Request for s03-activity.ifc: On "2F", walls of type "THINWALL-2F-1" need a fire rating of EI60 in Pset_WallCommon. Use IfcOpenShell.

First a look at what the model holds.

```python
import ifcopenshell
import ifcopenshell.util.element

model = ifcopenshell.open("s03-activity.ifc")
print(model.schema)
storey = next(s for s in model.by_type("IfcBuildingStorey") if s.Name == "2F")
walls = [e for e in ifcopenshell.util.element.get_decomposition(storey) if e.is_a("IfcWall")]
seen = {}
for e in walls:
    element_type = ifcopenshell.util.element.get_type(e)
    key = (element_type.Name if element_type != e and element_type else None, ifcopenshell.util.element.get_pset(e, "Pset_WallCommon", "FireRating"))
    seen[key] = seen.get(key, 0) + 1
for (name, value), count in sorted(seen.items(), key=str):
    print(count, "x", name, "|", value)
```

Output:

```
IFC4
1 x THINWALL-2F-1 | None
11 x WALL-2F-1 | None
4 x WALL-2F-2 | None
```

```python
import ifcopenshell
import ifcopenshell.api.pset
import ifcopenshell.util.element

model = ifcopenshell.open("s03-activity.ifc")

storey = next(s for s in model.by_type("IfcBuildingStorey") if s.Name == "2F")
walls = [e for e in ifcopenshell.util.element.get_decomposition(storey) if e.is_a("IfcWall")]

count = 0
for e in walls:
    element_type = ifcopenshell.util.element.get_type(e)
    if element_type in (None, e) or element_type.Name != "THINWALL-2F-1":
        continue
    # add_pset returns the element's existing set when there is one.
    pset = ifcopenshell.api.pset.add_pset(model, product=e, name="Pset_WallCommon")
    ifcopenshell.api.pset.edit_pset(model, pset=pset, properties={"FireRating": "EI60"})
    count += 1

print(count, "walls updated")

model.write("s03-activity_rev.ifc")
```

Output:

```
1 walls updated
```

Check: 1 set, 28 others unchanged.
